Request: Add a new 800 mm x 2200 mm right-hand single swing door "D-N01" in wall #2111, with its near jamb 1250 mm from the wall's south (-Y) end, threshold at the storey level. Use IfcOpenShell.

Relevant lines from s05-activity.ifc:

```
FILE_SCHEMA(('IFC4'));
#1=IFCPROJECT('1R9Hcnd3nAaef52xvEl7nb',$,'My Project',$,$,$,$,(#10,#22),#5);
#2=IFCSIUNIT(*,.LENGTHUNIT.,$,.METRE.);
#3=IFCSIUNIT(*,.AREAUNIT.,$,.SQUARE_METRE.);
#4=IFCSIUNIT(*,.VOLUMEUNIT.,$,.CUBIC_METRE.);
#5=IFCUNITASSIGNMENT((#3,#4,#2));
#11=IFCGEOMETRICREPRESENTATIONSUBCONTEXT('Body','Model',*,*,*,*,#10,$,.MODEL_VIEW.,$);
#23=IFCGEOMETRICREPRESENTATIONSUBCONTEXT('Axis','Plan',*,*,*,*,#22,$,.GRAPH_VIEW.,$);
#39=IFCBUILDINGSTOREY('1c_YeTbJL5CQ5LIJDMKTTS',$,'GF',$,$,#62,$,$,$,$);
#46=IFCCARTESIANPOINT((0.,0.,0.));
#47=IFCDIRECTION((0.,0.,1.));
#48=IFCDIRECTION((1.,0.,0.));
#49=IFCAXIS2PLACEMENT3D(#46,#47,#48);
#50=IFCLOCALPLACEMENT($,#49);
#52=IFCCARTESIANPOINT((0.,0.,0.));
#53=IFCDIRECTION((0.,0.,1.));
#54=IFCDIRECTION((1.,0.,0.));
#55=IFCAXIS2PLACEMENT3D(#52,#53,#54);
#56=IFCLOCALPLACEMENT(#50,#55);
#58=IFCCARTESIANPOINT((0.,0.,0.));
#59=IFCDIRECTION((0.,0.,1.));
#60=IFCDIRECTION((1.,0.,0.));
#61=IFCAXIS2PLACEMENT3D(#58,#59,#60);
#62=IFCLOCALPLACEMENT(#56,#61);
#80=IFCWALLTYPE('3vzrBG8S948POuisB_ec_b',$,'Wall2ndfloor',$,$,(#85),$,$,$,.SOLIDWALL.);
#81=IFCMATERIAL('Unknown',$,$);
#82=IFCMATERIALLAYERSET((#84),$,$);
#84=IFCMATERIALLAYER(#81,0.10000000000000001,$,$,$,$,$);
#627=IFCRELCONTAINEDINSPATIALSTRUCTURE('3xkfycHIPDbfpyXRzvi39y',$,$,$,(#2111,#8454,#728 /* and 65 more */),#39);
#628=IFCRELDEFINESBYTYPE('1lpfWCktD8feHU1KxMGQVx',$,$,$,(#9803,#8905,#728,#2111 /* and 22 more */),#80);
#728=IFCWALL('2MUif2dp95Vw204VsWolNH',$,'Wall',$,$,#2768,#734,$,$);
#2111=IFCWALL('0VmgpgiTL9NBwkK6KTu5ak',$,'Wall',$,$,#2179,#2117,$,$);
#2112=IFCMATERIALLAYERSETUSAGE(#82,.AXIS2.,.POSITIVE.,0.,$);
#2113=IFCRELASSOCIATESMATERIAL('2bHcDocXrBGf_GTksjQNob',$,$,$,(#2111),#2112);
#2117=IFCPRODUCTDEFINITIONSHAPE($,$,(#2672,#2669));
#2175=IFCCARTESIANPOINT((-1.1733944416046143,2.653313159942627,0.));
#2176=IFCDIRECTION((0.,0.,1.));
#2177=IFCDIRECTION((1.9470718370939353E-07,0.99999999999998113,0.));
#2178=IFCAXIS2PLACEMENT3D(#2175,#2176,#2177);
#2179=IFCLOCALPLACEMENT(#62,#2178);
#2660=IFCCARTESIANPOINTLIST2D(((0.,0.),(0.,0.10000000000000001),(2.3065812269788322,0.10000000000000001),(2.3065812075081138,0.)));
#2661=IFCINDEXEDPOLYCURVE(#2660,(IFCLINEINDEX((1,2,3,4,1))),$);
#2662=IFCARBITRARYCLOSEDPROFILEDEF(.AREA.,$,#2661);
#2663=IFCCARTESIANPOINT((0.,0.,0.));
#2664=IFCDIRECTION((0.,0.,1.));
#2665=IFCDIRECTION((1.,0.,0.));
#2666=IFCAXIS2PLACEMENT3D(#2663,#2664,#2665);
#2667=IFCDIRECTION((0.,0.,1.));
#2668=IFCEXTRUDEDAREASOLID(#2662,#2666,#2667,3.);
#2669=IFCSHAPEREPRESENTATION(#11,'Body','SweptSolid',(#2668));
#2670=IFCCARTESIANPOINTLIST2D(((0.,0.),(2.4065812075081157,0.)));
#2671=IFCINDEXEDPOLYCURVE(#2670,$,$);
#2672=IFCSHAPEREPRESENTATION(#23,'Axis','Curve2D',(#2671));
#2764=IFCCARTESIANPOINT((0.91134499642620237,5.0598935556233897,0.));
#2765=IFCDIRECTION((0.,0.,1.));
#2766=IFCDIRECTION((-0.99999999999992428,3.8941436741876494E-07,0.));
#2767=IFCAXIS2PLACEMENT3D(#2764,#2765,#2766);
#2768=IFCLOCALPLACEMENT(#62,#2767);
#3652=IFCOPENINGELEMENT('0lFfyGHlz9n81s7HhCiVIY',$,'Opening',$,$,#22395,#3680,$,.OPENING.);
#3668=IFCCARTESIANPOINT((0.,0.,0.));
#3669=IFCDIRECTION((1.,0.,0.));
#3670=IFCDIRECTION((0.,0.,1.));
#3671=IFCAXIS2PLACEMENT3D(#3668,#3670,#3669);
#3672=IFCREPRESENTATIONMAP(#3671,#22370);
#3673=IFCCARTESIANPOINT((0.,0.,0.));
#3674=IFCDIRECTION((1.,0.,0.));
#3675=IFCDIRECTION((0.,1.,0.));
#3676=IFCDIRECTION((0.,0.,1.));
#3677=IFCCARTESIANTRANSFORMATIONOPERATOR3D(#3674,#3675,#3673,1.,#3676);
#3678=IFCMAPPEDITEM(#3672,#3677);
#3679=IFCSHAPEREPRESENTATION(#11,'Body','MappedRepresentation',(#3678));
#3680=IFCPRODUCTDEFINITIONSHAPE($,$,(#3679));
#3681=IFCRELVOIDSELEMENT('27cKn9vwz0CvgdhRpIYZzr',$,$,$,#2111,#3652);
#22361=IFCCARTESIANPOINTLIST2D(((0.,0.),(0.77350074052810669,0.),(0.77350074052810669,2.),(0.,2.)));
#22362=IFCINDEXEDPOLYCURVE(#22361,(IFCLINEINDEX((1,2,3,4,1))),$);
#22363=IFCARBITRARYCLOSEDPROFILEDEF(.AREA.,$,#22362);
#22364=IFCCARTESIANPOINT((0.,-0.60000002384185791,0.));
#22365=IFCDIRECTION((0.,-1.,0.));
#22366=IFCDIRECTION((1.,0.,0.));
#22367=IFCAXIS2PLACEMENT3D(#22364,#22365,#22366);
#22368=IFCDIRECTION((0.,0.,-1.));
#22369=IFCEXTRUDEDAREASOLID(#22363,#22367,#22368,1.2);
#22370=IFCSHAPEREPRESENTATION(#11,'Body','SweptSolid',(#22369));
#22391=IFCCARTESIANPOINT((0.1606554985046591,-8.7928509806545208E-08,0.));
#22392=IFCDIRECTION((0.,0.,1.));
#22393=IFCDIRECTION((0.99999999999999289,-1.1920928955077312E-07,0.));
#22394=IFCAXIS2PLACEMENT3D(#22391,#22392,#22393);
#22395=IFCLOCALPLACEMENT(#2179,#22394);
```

```python
import numpy as np
import ifcopenshell
import ifcopenshell.api.feature
import ifcopenshell.api.geometry
import ifcopenshell.api.root
import ifcopenshell.api.spatial
import ifcopenshell.geom
import ifcopenshell.util.element
import ifcopenshell.util.placement
import ifcopenshell.util.representation
import ifcopenshell.util.shape
import ifcopenshell.util.unit

model = ifcopenshell.open("s05-activity.ifc")
unit_scale = ifcopenshell.util.unit.calculate_unit_scale(model)
settings = ifcopenshell.geom.settings()


def volume(element):
    """Net volume in cubic metres, openings subtracted."""
    shape = ifcopenshell.geom.create_shape(settings, element)
    return ifcopenshell.util.shape.get_volume(shape.geometry)


wall = model.by_id(2111)
storey = ifcopenshell.util.element.get_container(wall, ifc_class="IfcBuildingStorey")
context = ifcopenshell.util.representation.get_context(model, "Model", "Body", "MODEL_VIEW")
before = volume(wall)

width, height, from_end, sill = 0.8, 2.2, 1.25, 0.0  # metres

# The wall runs along its own X axis, and the end named is its -X end.
wall_shape = ifcopenshell.geom.create_shape(settings, wall)
x, y, z = ifcopenshell.util.shape.get_vertices(wall_shape.geometry).T
start = x.min() + from_end
face, thickness = float(y.min()), float(y.max() - y.min())
wall_matrix = ifcopenshell.util.placement.get_local_placement(wall.ObjectPlacement)
level = ifcopenshell.util.placement.get_local_placement(storey.ObjectPlacement)[2, 3]


def in_wall(x, y):
    """Placement at x, y metres in the wall's axes, at sill height."""
    matrix = wall_matrix.copy()
    matrix[:, 3] = wall_matrix @ np.array([x / unit_scale, y / unit_scale, 0.0, 1.0])
    matrix[2, 3] = level + sill / unit_scale
    return matrix


# Opening: a box that overshoots both wall faces by 50 mm.
opening = ifcopenshell.api.root.create_entity(model, ifc_class="IfcOpeningElement", predefined_type="OPENING")
box = ifcopenshell.api.geometry.add_wall_representation(
    model, context=context, length=width, height=height, thickness=thickness + 0.1
)
ifcopenshell.api.geometry.assign_representation(model, product=opening, representation=box)
ifcopenshell.api.geometry.edit_object_placement(model, product=opening, matrix=in_wall(start, face - 0.05), is_si=False)
ifcopenshell.api.feature.add_feature(model, feature=opening, element=wall)

door = ifcopenshell.api.root.create_entity(model, ifc_class="IfcDoor", name="D-N01", predefined_type="DOOR")
door.OverallWidth, door.OverallHeight = width / unit_scale, height / unit_scale
door.OperationType = "SINGLE_SWING_RIGHT"
body = ifcopenshell.api.geometry.add_door_representation(
    model,
    context=context,
    overall_width=door.OverallWidth,
    overall_height=door.OverallHeight,
    operation_type="SINGLE_SWING_RIGHT",
    lining_properties={"LiningDepth": thickness / unit_scale, "ThresholdDepth": thickness / unit_scale},
)
ifcopenshell.api.geometry.assign_representation(model, product=door, representation=body)
ifcopenshell.api.spatial.assign_container(model, products=[door], relating_structure=storey)
ifcopenshell.api.feature.add_filling(model, opening=opening, element=door)

# The lining spans the wall, so the door starts at the wall face.
ifcopenshell.api.geometry.edit_object_placement(model, product=door, matrix=in_wall(start, face), is_si=False)

after = volume(wall)

print(f"wall volume {before:.3f} -> {after:.3f} m3")

model.write("s05-activity-out.ifc")
```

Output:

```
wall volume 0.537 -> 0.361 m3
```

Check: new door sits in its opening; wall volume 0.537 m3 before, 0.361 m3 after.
